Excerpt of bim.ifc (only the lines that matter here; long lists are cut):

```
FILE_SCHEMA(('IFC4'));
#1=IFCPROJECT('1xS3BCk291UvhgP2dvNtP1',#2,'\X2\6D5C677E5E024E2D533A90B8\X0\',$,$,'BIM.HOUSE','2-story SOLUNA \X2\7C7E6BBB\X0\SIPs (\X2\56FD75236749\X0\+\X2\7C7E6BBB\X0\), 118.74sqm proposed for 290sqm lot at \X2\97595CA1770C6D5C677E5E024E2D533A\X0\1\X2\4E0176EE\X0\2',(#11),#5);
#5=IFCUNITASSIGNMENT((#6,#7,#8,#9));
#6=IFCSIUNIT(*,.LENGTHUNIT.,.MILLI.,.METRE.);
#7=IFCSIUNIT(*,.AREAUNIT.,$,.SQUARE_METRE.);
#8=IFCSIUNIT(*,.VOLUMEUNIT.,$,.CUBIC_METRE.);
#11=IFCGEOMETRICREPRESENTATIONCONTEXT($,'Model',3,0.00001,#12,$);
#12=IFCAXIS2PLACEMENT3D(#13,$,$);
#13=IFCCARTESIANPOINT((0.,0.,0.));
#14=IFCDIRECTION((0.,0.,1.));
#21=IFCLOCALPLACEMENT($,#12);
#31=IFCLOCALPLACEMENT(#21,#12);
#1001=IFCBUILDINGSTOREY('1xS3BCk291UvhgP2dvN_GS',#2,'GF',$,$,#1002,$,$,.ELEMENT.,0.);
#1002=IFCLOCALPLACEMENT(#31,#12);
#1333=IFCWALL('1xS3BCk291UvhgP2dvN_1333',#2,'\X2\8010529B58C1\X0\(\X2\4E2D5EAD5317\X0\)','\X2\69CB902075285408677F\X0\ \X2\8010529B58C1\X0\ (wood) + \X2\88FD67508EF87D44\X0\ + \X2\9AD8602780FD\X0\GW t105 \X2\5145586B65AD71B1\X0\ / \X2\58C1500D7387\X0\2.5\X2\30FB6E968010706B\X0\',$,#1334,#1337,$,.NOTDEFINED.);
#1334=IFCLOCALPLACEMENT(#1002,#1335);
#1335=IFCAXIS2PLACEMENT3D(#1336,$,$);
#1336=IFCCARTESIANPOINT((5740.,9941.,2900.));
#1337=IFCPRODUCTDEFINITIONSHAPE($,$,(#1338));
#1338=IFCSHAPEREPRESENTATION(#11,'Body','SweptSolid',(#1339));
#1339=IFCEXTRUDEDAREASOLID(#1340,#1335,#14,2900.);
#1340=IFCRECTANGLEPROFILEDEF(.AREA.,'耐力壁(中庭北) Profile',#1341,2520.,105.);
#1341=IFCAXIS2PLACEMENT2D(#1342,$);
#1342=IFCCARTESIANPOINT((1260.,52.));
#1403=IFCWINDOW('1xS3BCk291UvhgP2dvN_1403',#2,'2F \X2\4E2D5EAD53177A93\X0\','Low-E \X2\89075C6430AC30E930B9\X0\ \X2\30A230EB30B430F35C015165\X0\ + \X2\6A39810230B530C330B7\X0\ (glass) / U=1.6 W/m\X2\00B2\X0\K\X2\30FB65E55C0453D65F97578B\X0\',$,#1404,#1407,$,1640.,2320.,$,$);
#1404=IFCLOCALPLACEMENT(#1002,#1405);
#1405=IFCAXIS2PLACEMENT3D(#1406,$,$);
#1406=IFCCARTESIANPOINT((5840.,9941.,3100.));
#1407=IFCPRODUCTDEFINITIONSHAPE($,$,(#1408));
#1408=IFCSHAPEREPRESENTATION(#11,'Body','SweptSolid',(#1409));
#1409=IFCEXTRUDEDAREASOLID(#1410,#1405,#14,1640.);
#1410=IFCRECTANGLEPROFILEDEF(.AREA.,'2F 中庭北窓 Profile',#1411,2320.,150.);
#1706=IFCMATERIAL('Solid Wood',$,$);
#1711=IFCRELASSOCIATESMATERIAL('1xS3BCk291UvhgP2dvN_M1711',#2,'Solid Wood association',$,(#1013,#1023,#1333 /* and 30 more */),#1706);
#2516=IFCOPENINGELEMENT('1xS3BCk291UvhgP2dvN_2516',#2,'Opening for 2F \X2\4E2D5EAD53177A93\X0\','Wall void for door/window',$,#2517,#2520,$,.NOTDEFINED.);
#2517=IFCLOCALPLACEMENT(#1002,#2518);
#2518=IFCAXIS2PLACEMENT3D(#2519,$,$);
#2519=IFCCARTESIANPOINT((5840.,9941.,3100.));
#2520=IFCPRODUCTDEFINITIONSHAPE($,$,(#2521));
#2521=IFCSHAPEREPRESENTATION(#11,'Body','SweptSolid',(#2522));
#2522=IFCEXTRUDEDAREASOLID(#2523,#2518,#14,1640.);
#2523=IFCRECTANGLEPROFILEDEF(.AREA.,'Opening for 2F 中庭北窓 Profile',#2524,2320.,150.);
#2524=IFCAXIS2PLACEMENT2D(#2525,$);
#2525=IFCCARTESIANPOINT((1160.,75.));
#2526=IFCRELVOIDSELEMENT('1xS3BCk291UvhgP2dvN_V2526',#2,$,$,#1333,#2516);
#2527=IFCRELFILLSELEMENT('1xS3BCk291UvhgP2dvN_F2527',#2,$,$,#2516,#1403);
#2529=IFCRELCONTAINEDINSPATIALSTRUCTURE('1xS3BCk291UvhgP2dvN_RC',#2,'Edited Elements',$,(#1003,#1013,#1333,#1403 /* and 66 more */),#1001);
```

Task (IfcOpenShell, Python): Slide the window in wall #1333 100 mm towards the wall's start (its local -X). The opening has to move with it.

```python
import ifcopenshell
import ifcopenshell.api.geometry
import ifcopenshell.util.placement
import ifcopenshell.util.unit

model = ifcopenshell.open("bim.ifc")
unit_scale = ifcopenshell.util.unit.calculate_unit_scale(model)

window = model.by_guid("1xS3BCk291UvhgP2dvN_1403")
opening = window.FillsVoids[0].RelatingOpeningElement
wall = opening.VoidsElements[0].RelatingBuildingElement

wall_matrix = ifcopenshell.util.placement.get_local_placement(wall.ObjectPlacement)
shift = wall_matrix[:3, 0] * -0.1 / unit_scale
before = ifcopenshell.util.placement.get_local_placement(window.ObjectPlacement)[:3, 3].copy()

# The window is not placed relative to its opening, so move both.
for product in (opening, window):
    matrix = ifcopenshell.util.placement.get_local_placement(product.ObjectPlacement)
    matrix[:3, 3] += shift
    ifcopenshell.api.geometry.edit_object_placement(model, product=product, matrix=matrix, is_si=False)

after = ifcopenshell.util.placement.get_local_placement(window.ObjectPlacement)[:3, 3]
print("window moved by", (after - before).round(3) + 0.0)

model.write("bim-out.ifc")
```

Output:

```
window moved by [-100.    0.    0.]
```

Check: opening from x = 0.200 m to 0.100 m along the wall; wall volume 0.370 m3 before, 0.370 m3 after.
